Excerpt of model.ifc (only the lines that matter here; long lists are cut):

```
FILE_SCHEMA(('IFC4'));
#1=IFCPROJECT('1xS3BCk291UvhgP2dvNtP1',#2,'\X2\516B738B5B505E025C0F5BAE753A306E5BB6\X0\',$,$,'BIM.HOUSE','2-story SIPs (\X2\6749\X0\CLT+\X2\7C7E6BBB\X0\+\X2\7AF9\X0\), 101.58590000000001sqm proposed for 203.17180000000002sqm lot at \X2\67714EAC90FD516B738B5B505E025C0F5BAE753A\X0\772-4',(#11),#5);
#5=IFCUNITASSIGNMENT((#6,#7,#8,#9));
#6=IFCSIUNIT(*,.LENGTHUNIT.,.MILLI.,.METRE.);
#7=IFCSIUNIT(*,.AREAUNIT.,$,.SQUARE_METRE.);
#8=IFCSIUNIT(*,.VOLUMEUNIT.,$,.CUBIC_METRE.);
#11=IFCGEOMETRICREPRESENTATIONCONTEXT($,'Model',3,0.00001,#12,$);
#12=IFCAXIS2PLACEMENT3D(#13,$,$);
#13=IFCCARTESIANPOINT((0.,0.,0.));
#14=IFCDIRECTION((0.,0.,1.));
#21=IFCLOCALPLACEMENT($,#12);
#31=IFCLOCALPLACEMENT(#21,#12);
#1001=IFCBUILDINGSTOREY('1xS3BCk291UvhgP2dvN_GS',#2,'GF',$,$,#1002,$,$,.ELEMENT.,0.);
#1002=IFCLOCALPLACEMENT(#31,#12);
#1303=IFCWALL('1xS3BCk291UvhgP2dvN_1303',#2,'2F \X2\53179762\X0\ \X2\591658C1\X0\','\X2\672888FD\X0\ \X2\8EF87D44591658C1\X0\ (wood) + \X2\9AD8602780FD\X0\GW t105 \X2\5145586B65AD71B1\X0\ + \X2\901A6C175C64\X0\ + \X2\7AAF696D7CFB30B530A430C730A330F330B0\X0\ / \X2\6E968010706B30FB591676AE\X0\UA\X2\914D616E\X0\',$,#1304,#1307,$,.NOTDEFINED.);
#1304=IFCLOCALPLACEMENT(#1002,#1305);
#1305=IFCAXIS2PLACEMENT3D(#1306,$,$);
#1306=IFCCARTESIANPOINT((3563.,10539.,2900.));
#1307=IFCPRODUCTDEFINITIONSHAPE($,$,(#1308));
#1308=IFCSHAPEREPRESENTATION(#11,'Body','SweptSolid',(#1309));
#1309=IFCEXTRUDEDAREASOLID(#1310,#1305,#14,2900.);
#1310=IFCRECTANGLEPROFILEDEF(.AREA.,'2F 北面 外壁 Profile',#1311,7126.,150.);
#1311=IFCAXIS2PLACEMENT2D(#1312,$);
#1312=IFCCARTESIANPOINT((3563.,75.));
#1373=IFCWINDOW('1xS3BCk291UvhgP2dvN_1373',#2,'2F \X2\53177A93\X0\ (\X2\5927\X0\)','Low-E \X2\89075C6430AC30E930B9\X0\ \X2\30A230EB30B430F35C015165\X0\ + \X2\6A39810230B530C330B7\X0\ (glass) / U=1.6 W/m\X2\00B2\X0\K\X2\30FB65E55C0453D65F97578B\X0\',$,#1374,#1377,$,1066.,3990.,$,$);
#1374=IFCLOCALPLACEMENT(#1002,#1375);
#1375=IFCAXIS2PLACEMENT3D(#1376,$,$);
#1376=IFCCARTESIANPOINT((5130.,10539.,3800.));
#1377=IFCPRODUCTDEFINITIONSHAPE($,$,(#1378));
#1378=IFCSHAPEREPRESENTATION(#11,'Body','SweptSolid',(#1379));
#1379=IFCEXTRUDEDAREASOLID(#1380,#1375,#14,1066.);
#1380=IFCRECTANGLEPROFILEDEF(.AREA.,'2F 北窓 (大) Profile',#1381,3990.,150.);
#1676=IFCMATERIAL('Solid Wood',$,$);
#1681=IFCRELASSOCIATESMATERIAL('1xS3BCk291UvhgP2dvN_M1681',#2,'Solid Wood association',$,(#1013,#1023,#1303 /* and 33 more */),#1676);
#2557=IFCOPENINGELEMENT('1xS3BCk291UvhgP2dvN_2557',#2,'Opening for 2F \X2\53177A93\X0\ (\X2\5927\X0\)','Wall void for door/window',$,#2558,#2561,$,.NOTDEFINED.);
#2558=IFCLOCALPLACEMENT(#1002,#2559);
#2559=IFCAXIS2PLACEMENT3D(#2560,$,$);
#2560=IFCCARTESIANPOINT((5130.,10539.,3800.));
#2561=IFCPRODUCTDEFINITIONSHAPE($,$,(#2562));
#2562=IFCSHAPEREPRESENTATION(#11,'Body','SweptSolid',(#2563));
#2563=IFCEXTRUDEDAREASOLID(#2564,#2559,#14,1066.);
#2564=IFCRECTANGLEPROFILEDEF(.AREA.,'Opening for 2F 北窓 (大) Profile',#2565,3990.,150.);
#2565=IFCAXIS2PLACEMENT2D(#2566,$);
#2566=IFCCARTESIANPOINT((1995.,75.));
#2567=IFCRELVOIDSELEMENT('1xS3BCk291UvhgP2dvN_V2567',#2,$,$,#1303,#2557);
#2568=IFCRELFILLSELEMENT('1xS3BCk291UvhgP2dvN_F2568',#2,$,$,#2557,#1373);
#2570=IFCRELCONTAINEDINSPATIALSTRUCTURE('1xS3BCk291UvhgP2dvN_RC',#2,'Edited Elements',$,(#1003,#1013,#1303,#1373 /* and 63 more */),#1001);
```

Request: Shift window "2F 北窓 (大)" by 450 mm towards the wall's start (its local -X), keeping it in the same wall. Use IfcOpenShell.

```python
import ifcopenshell
import ifcopenshell.api.geometry
import ifcopenshell.util.placement

model = ifcopenshell.open("model.ifc")

window = model.by_guid("1xS3BCk291UvhgP2dvN_1373")
opening = window.FillsVoids[0].RelatingOpeningElement
wall = opening.VoidsElements[0].RelatingBuildingElement

wall_matrix = ifcopenshell.util.placement.get_local_placement(wall.ObjectPlacement)
shift = wall_matrix[:3, 0] * -450.0
before = ifcopenshell.util.placement.get_local_placement(window.ObjectPlacement)[:3, 3].copy()

# The window is not placed relative to its opening, so move both.
for product in (opening, window):
    matrix = ifcopenshell.util.placement.get_local_placement(product.ObjectPlacement)
    matrix[:3, 3] += shift
    ifcopenshell.api.geometry.edit_object_placement(model, product=product, matrix=matrix, is_si=False)

after = ifcopenshell.util.placement.get_local_placement(window.ObjectPlacement)[:3, 3]
print("window moved by", (after - before).round(3) + 0.0)

model.write("model-out.ifc")
```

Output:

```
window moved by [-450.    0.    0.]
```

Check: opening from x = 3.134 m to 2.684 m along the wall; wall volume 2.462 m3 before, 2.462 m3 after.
